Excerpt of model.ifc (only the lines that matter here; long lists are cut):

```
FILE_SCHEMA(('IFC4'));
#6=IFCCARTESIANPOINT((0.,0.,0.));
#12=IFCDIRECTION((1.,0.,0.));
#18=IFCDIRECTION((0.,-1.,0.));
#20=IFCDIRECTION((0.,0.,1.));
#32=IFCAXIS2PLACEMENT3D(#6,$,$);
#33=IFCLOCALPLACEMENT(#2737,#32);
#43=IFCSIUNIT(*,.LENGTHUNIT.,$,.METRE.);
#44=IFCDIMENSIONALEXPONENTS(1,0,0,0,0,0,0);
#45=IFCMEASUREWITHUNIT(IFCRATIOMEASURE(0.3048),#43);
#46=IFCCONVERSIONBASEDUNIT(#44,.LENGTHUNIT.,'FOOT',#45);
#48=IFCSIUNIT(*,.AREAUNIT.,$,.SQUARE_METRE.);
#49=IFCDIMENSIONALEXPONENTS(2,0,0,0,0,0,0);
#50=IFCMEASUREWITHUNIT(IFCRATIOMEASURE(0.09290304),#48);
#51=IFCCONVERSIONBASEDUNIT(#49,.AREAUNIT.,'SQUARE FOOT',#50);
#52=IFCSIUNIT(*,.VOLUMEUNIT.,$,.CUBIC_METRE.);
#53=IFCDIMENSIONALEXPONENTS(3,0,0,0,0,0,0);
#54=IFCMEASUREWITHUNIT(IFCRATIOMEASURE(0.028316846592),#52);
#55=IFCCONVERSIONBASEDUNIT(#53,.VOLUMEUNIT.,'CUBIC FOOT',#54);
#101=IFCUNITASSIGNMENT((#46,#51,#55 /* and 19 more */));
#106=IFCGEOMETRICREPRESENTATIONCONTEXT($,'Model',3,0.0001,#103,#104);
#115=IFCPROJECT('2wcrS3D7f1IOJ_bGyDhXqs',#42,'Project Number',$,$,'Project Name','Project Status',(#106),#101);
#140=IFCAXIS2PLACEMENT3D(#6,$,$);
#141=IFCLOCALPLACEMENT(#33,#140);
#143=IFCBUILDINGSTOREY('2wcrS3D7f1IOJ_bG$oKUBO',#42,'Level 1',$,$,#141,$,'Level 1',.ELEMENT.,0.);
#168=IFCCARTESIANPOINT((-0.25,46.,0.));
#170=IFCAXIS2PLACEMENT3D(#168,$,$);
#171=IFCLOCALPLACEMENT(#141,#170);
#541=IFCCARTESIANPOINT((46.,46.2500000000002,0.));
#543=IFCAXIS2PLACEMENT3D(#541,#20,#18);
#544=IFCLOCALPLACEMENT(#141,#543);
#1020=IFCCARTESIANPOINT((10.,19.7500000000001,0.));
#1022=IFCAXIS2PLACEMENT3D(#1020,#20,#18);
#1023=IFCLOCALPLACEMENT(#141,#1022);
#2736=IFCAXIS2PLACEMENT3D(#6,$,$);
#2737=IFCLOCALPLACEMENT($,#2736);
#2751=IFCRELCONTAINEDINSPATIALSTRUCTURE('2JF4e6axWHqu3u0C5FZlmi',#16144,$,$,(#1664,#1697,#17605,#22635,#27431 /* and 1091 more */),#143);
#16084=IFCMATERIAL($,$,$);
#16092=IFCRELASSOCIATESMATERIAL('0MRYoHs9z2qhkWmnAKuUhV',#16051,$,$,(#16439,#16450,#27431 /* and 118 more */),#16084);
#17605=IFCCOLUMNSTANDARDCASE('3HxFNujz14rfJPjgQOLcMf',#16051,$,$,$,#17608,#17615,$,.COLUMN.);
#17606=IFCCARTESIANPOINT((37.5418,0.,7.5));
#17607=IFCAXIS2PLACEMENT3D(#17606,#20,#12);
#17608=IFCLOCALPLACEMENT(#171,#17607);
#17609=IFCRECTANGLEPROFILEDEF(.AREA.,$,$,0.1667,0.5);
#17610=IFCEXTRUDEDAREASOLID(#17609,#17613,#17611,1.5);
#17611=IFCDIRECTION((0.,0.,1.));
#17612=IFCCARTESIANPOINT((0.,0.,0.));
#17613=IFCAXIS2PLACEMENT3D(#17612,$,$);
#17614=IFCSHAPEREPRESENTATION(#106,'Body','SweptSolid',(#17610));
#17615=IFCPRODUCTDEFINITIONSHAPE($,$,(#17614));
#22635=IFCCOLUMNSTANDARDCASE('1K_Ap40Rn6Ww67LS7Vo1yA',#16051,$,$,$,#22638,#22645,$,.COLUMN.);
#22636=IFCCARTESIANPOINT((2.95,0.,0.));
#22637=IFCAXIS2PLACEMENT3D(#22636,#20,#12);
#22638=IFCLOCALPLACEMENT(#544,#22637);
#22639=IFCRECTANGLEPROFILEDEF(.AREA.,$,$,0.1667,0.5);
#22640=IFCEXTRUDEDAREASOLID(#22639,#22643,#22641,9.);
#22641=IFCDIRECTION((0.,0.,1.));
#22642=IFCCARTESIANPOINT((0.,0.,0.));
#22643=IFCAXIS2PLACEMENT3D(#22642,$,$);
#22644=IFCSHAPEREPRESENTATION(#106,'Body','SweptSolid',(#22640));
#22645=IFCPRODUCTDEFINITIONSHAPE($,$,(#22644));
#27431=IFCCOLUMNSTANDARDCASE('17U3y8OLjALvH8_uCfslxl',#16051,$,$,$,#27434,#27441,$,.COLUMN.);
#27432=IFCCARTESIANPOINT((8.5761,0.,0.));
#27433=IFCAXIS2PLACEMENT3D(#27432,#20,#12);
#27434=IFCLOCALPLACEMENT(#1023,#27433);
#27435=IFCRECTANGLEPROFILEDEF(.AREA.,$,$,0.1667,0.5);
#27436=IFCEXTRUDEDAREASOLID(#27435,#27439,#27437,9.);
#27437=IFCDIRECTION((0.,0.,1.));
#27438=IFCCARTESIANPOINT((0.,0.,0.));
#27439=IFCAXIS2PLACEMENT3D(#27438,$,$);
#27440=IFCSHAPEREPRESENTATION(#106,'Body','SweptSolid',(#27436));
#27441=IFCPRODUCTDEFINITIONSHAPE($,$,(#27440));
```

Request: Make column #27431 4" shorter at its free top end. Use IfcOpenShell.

```python
import ifcopenshell
import ifcopenshell.util.unit

model = ifcopenshell.open("model.ifc")
unit_scale = ifcopenshell.util.unit.calculate_unit_scale(model)

member = model.by_id(27431)
change = -4 * 0.0254 / unit_scale

# The extrusion runs towards the end named, so only its depth changes.
body = next(r for r in member.Representation.Representations if r.RepresentationIdentifier == "Body")
solid = body.Items[0]
old_length = solid.Depth
solid.Depth += change

print(f"length {old_length:g} -> {solid.Depth:g}")

model.write("model_rev.ifc")
```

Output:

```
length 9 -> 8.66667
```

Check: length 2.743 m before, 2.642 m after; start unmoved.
